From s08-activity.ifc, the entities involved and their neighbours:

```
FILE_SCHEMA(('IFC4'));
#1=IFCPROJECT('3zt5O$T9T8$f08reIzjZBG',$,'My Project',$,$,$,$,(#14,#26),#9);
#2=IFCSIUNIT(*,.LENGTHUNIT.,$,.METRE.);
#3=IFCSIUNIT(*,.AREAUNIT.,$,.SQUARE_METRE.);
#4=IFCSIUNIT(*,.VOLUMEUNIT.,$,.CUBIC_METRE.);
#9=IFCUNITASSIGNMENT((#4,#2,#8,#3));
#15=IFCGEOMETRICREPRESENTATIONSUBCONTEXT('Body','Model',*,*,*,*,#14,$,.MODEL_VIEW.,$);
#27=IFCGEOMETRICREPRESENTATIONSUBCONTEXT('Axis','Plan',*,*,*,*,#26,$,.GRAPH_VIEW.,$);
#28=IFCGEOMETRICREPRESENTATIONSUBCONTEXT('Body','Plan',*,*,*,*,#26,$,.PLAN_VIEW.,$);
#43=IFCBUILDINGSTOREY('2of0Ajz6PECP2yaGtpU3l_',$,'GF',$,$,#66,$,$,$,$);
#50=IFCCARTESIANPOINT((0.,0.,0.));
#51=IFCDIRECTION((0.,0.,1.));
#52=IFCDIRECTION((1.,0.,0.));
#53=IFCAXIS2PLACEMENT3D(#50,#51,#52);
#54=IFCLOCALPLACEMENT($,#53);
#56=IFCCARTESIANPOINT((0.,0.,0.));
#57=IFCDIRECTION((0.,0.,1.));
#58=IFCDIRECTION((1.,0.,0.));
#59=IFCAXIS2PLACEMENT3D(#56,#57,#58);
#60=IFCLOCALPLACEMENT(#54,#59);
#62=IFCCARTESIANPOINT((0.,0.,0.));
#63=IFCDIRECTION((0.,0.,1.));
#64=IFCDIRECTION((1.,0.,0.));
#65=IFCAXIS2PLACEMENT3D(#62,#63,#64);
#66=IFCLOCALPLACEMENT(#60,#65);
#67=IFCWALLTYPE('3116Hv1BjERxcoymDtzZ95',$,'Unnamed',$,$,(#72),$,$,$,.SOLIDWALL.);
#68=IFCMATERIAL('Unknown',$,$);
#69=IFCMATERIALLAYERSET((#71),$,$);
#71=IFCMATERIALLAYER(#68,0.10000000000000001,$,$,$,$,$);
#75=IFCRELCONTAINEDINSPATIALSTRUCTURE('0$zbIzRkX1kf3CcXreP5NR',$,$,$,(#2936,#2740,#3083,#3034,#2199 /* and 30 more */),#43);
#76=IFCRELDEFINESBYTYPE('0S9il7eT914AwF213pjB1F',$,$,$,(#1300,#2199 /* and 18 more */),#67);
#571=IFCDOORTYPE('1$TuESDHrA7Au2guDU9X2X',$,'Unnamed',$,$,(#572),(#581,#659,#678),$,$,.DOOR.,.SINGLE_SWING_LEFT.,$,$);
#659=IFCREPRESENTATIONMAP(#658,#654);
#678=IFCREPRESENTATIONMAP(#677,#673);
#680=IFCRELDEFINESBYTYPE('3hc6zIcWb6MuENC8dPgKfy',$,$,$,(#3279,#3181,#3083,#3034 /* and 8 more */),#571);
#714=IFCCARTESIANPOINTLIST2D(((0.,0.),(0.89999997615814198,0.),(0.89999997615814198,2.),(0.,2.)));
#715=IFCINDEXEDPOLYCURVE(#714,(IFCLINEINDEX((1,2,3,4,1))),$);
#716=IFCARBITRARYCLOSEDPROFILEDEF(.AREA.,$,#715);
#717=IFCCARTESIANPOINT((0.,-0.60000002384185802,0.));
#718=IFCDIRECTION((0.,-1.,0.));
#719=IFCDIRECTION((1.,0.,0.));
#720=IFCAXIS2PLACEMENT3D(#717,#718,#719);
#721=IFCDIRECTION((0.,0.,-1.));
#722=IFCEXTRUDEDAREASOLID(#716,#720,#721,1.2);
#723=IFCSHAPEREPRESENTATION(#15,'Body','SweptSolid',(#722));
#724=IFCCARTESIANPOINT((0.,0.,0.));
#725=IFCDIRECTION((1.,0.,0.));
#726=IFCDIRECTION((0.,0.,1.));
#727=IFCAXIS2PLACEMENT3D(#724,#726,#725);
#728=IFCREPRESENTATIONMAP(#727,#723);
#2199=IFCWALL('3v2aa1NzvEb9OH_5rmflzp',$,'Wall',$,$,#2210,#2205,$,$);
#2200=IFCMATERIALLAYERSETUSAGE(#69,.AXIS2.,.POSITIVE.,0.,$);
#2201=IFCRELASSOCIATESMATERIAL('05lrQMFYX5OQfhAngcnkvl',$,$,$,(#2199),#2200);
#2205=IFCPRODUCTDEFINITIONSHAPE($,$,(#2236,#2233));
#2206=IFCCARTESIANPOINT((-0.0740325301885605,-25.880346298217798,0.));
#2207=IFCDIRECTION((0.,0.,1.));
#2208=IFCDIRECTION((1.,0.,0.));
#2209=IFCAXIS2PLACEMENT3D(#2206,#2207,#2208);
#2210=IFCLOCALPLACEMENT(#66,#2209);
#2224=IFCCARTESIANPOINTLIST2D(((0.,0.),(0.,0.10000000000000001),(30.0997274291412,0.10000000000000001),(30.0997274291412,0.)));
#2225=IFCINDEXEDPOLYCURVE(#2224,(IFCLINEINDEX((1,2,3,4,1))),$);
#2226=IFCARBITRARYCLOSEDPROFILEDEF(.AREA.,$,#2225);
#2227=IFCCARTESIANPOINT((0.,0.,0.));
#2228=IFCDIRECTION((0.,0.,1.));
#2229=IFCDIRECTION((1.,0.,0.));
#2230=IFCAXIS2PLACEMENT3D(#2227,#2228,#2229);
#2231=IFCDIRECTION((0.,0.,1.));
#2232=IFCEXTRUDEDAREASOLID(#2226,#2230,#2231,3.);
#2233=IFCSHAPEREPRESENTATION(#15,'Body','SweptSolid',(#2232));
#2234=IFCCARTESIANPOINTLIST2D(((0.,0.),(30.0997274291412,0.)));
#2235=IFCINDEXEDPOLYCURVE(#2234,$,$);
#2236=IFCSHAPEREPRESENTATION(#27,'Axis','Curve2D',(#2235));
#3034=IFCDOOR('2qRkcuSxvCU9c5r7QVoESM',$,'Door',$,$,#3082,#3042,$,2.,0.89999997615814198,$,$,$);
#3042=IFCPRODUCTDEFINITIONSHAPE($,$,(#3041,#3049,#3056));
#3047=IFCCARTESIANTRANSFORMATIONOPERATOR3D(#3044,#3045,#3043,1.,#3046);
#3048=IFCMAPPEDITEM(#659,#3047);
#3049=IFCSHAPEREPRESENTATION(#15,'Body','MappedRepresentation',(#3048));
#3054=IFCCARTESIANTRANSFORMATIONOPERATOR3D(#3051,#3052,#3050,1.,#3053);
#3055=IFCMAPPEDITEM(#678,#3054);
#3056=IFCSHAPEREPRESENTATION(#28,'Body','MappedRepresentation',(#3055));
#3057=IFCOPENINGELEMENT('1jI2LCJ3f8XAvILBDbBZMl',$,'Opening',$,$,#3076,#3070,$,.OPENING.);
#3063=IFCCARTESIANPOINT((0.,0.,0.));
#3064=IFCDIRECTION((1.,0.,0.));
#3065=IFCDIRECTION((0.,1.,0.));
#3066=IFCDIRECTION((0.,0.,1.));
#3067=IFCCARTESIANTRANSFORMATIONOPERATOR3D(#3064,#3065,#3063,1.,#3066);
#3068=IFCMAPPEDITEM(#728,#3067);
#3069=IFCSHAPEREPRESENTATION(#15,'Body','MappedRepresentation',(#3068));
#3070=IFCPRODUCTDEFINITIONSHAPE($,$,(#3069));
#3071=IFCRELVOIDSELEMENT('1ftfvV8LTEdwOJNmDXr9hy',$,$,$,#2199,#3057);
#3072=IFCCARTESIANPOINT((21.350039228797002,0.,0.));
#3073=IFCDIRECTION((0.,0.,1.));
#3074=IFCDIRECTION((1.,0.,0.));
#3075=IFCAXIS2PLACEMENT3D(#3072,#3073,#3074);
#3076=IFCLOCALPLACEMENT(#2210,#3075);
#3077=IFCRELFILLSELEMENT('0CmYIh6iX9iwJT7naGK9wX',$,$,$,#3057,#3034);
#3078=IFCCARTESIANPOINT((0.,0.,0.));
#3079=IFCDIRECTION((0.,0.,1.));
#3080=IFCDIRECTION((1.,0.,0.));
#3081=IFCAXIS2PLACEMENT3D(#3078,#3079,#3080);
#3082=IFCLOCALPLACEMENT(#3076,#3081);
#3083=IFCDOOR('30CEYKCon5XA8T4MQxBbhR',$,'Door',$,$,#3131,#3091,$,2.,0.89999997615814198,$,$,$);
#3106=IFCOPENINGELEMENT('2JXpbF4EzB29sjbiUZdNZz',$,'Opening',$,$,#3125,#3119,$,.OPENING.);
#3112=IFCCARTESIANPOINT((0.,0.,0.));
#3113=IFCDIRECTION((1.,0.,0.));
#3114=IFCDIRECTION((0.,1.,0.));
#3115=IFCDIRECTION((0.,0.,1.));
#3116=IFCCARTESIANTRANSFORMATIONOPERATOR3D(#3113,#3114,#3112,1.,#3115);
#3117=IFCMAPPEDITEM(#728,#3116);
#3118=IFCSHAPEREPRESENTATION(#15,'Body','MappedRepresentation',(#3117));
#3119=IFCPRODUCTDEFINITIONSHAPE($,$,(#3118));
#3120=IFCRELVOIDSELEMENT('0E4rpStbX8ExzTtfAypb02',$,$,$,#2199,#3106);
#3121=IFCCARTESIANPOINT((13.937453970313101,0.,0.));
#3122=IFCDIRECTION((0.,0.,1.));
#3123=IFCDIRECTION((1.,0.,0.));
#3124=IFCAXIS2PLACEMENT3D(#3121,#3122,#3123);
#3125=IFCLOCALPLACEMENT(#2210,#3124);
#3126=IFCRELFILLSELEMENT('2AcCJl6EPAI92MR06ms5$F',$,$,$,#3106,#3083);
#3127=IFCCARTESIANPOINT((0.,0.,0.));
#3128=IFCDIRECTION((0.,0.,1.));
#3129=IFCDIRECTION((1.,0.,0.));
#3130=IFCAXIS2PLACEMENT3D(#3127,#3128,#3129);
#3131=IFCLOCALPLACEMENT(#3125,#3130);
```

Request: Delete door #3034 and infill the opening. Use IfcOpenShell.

```python
import ifcopenshell
import ifcopenshell.api.feature
import ifcopenshell.api.root
import ifcopenshell.geom
import ifcopenshell.util.shape

model = ifcopenshell.open("s08-activity.ifc")
settings = ifcopenshell.geom.settings()


def volume(element):
    """Net volume in cubic metres, openings subtracted."""
    shape = ifcopenshell.geom.create_shape(settings, element)
    return ifcopenshell.util.shape.get_volume(shape.geometry)


door = model.by_guid("2qRkcuSxvCU9c5r7QVoESM")
opening = door.FillsVoids[0].RelatingOpeningElement
wall = opening.VoidsElements[0].RelatingBuildingElement
before = volume(wall)

ifcopenshell.api.root.remove_product(model, product=door)
ifcopenshell.api.feature.remove_feature(model, feature=opening)

after = volume(wall)

print(f"wall volume {before:.3f} -> {after:.3f} m3")

model.write("s08-activity_rev.ifc")
```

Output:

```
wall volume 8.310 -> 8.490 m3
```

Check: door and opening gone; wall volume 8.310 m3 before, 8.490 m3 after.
